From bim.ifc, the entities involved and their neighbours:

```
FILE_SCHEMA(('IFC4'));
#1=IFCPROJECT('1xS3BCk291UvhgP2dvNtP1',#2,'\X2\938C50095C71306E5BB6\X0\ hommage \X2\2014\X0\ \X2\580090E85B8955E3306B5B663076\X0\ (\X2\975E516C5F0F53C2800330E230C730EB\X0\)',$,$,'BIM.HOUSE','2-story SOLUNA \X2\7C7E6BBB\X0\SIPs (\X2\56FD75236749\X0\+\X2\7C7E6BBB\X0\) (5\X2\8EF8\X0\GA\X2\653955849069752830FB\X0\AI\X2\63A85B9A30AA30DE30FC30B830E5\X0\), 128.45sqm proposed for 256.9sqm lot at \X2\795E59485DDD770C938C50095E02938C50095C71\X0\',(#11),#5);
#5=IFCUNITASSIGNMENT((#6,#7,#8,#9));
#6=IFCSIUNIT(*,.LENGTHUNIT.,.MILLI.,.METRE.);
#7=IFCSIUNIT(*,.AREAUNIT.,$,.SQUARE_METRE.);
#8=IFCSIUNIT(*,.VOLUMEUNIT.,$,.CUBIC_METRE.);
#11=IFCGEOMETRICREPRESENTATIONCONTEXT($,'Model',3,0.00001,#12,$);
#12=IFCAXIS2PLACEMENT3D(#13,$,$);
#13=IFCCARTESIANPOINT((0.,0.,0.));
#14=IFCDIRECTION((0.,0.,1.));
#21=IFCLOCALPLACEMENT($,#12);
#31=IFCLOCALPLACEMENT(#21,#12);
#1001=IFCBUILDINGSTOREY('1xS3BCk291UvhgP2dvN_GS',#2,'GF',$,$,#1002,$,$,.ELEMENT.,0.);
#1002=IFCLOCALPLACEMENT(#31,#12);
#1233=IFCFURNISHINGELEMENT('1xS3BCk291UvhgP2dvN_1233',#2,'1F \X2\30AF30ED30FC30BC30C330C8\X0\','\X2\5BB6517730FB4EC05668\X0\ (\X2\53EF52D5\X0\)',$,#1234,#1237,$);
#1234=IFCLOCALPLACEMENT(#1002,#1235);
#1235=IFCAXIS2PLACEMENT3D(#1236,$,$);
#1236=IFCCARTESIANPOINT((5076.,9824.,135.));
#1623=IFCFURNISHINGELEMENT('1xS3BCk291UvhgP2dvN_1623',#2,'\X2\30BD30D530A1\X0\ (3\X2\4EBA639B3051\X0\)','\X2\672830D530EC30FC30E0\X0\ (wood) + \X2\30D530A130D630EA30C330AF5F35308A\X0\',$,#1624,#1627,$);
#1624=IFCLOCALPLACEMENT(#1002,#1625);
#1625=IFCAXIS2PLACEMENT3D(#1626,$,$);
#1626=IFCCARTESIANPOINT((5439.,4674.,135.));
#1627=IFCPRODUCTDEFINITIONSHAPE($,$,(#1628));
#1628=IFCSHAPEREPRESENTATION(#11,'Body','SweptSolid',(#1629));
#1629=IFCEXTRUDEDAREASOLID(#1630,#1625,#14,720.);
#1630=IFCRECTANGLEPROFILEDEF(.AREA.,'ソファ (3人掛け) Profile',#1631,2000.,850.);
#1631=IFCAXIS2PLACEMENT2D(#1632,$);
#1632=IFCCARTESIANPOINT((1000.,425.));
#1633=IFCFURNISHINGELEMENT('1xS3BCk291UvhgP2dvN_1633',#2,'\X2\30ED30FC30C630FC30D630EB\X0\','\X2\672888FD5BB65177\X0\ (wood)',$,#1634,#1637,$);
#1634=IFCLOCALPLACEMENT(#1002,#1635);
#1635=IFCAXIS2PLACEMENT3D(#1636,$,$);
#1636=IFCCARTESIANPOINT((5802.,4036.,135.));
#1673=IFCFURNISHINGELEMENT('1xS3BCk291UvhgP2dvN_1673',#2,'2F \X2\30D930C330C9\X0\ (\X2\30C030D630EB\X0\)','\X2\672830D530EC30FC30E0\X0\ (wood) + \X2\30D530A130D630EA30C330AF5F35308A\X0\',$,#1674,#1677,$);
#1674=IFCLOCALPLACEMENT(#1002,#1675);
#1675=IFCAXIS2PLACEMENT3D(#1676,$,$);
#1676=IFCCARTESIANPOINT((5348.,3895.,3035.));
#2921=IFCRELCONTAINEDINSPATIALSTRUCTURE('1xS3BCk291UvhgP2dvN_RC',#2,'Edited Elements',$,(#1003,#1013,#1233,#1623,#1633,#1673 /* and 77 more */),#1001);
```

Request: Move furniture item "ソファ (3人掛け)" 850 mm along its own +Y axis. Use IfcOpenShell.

```python
import ifcopenshell
import ifcopenshell.api.geometry
import ifcopenshell.util.placement

model = ifcopenshell.open("bim.ifc")

item = model.by_guid("1xS3BCk291UvhgP2dvN_1623")
matrix = ifcopenshell.util.placement.get_local_placement(item.ObjectPlacement)
matrix[:3, 3] += matrix[:3, 1] * 850.0
ifcopenshell.api.geometry.edit_object_placement(model, product=item, matrix=matrix, is_si=False)

print(ifcopenshell.util.placement.get_local_placement(item.ObjectPlacement).round(3) + 0.0)

model.write("bim_v2.ifc")
```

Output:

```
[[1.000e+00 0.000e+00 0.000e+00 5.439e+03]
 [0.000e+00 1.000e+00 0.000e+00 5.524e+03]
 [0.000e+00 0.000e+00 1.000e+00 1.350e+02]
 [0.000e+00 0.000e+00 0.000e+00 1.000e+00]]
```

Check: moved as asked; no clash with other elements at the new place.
